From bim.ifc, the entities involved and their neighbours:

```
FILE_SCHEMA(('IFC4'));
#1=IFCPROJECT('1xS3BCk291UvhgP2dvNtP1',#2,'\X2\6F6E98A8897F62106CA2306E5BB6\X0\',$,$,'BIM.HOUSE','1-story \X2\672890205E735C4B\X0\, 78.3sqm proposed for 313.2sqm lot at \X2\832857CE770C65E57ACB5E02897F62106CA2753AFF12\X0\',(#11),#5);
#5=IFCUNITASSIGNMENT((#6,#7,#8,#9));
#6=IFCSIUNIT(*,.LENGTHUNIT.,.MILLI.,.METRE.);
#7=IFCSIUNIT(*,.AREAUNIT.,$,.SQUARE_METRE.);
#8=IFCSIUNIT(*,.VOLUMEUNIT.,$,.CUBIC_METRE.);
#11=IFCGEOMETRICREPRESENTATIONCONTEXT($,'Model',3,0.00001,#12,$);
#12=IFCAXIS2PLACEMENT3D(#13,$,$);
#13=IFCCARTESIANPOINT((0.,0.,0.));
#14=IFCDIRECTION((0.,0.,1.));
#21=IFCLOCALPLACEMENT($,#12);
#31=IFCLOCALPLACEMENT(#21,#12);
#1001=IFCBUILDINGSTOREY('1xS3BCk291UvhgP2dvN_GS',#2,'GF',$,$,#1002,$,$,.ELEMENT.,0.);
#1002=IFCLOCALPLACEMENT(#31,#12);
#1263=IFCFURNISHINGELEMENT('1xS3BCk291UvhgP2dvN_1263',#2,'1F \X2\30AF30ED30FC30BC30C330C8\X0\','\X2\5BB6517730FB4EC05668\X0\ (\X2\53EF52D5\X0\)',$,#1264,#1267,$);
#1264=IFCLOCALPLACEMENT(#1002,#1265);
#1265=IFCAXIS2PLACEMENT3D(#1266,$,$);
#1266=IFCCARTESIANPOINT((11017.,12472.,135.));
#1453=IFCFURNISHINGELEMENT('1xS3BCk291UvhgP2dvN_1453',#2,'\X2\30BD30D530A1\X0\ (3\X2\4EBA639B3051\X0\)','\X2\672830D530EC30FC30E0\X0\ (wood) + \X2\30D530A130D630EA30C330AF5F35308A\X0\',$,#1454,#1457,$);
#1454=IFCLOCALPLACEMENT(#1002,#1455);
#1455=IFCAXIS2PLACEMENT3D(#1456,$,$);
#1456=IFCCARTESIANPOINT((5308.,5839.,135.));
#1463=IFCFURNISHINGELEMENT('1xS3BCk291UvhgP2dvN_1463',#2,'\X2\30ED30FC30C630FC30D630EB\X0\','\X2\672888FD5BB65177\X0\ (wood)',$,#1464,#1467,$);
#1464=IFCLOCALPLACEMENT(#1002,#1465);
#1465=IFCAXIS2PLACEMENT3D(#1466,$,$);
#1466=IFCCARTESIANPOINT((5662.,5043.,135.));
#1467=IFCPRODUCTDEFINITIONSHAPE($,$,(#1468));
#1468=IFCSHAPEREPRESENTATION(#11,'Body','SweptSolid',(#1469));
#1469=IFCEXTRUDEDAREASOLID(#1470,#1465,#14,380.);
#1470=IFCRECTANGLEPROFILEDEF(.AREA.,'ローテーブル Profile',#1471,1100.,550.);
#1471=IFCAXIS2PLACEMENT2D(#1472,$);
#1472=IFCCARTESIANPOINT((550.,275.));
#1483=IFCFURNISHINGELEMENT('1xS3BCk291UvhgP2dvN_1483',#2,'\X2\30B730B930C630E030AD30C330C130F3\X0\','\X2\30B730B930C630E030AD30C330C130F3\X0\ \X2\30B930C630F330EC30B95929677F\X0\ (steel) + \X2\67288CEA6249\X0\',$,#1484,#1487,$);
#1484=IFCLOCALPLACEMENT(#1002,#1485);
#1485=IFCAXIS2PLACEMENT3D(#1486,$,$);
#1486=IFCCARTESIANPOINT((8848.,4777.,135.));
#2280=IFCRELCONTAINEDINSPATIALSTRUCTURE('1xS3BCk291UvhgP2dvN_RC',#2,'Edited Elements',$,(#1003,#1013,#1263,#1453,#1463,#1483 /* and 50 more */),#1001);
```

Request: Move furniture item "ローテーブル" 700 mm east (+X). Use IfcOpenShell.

```python
import ifcopenshell
import ifcopenshell.api.geometry
import ifcopenshell.util.placement
import ifcopenshell.util.unit

model = ifcopenshell.open("bim.ifc")
unit_scale = ifcopenshell.util.unit.calculate_unit_scale(model)

item = model.by_guid("1xS3BCk291UvhgP2dvN_1463")
matrix = ifcopenshell.util.placement.get_local_placement(item.ObjectPlacement)
matrix[0, 3] += 0.7 / unit_scale
ifcopenshell.api.geometry.edit_object_placement(model, product=item, matrix=matrix, is_si=False)

print(ifcopenshell.util.placement.get_local_placement(item.ObjectPlacement).round(3) + 0.0)

model.write("bim_rev.ifc")
```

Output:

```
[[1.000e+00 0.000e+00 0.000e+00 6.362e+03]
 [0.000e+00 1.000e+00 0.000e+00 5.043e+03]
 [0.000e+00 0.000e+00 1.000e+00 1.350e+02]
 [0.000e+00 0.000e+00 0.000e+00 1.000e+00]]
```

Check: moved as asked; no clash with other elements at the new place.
